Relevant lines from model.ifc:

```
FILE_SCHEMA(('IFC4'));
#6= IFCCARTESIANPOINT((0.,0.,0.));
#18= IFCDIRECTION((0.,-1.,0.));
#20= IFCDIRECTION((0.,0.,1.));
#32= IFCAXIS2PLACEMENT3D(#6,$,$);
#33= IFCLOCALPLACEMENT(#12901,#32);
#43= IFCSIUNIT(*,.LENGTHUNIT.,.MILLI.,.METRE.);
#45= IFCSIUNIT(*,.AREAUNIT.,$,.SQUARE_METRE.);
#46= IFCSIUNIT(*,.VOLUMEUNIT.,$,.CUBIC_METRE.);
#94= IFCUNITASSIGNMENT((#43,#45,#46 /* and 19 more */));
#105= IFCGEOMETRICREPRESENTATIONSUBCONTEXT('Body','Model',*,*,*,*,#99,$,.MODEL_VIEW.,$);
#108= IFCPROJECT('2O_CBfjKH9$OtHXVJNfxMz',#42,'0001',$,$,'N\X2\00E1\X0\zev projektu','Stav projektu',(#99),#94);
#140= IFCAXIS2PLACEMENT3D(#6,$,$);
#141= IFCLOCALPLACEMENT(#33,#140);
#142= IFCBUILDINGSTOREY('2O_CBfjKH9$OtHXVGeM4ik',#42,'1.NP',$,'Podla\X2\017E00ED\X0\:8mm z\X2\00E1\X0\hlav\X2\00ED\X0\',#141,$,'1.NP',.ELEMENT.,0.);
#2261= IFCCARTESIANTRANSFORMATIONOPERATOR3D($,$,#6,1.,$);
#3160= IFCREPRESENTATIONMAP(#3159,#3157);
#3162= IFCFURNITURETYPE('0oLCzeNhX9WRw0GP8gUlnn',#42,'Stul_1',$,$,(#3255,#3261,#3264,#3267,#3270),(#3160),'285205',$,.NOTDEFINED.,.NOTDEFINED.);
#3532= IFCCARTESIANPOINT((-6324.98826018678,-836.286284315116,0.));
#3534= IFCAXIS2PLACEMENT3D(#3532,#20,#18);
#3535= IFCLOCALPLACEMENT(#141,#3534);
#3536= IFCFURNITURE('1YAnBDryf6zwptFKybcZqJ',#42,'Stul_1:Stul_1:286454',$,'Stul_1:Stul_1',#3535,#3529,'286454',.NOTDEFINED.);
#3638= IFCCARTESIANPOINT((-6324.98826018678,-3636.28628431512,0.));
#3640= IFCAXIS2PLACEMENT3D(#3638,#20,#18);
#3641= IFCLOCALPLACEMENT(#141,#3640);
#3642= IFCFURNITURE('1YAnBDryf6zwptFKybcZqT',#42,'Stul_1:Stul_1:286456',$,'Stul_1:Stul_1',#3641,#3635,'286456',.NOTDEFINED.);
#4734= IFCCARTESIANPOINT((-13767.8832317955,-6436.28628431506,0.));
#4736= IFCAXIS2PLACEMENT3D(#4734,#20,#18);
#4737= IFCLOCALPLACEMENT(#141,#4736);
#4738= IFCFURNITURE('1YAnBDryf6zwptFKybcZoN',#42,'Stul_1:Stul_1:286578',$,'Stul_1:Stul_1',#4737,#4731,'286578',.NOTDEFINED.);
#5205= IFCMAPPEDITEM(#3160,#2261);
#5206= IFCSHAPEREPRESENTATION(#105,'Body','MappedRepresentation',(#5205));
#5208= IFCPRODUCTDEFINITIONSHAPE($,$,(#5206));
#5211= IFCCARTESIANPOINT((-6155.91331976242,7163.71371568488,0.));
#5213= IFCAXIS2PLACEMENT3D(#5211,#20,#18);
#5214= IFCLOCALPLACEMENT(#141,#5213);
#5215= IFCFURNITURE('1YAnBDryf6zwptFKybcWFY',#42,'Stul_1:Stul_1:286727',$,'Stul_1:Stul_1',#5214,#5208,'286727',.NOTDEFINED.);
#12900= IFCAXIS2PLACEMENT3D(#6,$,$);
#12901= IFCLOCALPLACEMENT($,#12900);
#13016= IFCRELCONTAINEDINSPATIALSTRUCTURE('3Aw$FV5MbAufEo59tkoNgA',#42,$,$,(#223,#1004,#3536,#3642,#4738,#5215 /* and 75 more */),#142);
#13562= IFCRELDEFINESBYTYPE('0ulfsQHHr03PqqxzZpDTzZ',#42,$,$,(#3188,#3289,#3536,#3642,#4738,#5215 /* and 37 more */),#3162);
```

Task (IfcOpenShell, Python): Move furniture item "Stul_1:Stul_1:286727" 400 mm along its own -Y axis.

```python
import ifcopenshell
import ifcopenshell.api.geometry
import ifcopenshell.util.placement
import ifcopenshell.util.unit

model = ifcopenshell.open("model.ifc")
unit_scale = ifcopenshell.util.unit.calculate_unit_scale(model)

item = model.by_id(5215)
matrix = ifcopenshell.util.placement.get_local_placement(item.ObjectPlacement)
matrix[:3, 3] -= matrix[:3, 1] * 0.4 / unit_scale
ifcopenshell.api.geometry.edit_object_placement(model, product=item, matrix=matrix, is_si=False)

print(ifcopenshell.util.placement.get_local_placement(item.ObjectPlacement).round(3) + 0.0)

model.write("model_updated.ifc")
```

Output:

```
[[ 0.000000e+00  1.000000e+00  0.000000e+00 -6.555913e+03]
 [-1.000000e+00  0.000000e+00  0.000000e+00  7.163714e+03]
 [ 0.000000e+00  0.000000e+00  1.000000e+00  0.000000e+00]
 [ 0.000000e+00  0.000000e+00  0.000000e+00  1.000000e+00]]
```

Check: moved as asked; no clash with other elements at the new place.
